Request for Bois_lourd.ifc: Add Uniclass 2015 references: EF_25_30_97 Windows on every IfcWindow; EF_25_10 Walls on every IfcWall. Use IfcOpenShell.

First a look at what the model holds.

```python
import ifcopenshell

model = ifcopenshell.open("Bois_lourd.ifc")
print(model.schema)
print("classifications:", [c.Name for c in model.by_type("IfcClassification")])
for ifc_class in ("IfcDoor", "IfcRoof", "IfcStair", "IfcWall", "IfcWindow"):
    print(ifc_class, len(model.by_type(ifc_class)))
```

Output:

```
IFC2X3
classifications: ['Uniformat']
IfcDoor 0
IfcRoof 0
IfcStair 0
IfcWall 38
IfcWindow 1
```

```python
import ifcopenshell
import ifcopenshell.api.classification

model = ifcopenshell.open("Bois_lourd.ifc")

# IFC2X3 requires Source and Edition and has no link from the project to the system.
system = model.create_entity("IfcClassification", Source="NBS", Edition="2015", Name="Uniclass 2015")

codes = {
    "IfcWindow": ("EF_25_30_97", "Windows"),
    "IfcWall": ("EF_25_10", "Walls"),
}
for ifc_class, (code, name) in codes.items():
    products = model.by_type(ifc_class)
    ifcopenshell.api.classification.add_reference(
        model, products=products, classification=system, identification=code, name=name
    )
    print(code, len(products))

model.write("Bois_lourd_rev.ifc")
```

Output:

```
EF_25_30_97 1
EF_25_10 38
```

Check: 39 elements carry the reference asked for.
